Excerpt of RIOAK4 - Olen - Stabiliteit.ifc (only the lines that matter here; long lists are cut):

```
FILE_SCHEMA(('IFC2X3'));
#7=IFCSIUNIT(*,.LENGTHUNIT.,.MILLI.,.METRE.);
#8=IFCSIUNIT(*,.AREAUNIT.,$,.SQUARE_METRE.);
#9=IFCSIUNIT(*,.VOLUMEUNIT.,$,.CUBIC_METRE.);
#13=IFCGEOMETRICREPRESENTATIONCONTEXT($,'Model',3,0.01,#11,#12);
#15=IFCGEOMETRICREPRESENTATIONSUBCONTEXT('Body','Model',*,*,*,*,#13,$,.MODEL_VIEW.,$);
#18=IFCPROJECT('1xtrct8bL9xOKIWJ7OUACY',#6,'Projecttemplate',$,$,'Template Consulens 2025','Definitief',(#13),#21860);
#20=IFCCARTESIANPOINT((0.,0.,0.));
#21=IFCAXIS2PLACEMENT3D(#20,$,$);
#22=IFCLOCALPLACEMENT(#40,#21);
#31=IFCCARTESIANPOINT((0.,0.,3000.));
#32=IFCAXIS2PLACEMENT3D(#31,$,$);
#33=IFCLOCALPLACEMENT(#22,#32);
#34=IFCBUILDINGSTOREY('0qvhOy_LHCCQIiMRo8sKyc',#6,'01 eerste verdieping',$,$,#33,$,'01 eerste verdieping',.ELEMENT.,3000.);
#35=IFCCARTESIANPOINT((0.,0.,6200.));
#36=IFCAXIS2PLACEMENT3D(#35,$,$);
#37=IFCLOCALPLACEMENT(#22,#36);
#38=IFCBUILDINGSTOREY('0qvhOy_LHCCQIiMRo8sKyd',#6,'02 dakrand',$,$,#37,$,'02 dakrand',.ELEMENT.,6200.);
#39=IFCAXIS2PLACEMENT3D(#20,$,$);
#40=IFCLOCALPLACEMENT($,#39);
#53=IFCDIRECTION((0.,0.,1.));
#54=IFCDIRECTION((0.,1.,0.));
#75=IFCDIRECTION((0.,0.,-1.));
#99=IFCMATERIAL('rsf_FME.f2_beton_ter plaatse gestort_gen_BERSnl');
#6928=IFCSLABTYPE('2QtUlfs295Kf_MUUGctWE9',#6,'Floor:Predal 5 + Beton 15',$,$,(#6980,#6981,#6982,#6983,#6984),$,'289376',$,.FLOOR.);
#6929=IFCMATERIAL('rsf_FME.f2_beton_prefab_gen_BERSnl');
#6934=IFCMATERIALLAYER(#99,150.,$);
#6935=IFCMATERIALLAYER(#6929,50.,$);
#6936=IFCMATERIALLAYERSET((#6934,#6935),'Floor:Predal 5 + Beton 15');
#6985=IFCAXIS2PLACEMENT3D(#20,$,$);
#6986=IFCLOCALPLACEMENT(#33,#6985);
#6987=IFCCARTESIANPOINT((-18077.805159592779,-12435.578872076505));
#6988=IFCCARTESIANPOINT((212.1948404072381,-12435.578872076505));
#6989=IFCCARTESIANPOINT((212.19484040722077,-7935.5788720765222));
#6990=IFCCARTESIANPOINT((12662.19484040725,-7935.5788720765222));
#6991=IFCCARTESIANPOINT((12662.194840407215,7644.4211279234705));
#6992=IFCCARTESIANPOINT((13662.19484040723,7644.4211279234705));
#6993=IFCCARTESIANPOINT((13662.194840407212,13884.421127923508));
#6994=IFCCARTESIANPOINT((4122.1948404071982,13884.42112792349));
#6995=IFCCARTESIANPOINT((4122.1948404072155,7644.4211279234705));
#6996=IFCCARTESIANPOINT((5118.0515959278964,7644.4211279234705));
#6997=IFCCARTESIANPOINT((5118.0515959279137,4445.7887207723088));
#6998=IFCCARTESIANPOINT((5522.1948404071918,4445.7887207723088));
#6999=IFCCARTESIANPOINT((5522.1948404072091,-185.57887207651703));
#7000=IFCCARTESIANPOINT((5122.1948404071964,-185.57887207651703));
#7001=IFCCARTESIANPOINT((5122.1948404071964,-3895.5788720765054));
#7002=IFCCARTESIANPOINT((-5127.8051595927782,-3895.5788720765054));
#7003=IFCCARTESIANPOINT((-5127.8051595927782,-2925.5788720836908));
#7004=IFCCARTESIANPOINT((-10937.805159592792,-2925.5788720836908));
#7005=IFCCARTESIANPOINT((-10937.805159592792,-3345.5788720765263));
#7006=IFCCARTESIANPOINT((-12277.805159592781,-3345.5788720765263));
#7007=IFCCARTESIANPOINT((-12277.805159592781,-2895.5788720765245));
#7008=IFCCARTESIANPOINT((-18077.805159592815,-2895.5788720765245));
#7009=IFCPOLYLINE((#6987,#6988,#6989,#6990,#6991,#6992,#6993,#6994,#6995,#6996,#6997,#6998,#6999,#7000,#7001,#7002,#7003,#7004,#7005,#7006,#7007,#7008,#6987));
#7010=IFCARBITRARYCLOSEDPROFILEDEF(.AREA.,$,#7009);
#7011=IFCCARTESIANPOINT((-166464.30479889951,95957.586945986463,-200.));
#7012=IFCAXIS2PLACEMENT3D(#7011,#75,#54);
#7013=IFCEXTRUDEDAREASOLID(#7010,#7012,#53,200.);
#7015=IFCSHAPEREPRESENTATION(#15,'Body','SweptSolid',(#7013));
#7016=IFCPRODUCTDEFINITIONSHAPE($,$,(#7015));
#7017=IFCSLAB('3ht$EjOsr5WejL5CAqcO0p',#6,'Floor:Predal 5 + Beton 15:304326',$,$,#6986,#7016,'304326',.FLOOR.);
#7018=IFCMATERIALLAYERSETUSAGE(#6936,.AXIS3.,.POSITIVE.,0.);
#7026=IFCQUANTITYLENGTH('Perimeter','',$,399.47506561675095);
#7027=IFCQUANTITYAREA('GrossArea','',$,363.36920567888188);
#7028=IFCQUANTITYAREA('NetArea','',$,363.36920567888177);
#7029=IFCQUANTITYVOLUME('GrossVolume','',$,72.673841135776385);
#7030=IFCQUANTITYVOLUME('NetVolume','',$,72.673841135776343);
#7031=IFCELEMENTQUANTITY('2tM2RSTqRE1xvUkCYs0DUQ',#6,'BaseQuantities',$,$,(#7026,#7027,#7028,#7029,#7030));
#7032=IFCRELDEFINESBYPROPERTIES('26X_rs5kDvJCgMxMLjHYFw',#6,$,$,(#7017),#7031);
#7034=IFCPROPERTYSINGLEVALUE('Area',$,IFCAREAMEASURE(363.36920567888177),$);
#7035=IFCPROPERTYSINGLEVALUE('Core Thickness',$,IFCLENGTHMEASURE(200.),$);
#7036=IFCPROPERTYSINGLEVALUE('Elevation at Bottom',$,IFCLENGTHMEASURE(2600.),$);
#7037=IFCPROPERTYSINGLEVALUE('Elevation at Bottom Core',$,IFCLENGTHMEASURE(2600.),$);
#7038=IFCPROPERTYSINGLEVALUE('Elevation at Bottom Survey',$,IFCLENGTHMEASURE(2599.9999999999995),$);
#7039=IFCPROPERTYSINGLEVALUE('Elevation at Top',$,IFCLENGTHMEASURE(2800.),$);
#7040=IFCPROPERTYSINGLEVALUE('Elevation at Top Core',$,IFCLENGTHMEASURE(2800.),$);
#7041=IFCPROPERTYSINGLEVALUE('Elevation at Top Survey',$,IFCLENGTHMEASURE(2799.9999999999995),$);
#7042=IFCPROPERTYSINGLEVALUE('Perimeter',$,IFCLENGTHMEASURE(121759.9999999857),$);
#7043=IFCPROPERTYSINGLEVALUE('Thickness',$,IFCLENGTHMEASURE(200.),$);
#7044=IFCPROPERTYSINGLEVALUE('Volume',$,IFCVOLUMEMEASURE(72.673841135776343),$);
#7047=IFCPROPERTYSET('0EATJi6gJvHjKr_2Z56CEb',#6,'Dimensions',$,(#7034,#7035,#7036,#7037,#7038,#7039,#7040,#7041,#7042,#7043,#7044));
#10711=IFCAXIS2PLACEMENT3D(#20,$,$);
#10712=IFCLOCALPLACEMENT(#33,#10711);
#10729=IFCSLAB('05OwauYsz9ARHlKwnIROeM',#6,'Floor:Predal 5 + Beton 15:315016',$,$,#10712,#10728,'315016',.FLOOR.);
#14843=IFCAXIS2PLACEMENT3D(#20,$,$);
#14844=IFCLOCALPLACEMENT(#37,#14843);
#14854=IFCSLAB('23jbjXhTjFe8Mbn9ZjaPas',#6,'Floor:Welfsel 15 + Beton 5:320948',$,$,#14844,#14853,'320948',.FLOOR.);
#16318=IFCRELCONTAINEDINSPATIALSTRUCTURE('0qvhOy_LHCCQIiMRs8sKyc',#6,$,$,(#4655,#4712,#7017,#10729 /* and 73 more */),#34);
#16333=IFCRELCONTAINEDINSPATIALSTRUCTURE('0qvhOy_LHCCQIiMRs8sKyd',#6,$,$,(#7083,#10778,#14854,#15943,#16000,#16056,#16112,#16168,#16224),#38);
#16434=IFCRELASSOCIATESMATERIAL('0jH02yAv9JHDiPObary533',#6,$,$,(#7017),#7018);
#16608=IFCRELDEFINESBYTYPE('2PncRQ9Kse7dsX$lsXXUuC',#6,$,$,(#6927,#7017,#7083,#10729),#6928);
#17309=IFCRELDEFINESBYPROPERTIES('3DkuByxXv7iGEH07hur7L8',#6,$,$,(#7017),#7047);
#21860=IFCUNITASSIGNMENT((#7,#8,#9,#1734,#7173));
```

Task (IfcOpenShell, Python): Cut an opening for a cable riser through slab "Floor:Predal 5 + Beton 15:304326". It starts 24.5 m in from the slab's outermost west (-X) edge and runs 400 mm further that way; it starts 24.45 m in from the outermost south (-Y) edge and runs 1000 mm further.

```python
import numpy as np
import ifcopenshell
import ifcopenshell.api.feature
import ifcopenshell.api.geometry
import ifcopenshell.api.pset
import ifcopenshell.api.root
import ifcopenshell.geom
import ifcopenshell.util.element
import ifcopenshell.util.placement
import ifcopenshell.util.representation
import ifcopenshell.util.shape
import ifcopenshell.util.unit

model = ifcopenshell.open("RIOAK4 - Olen - Stabiliteit.ifc")
unit_scale = ifcopenshell.util.unit.calculate_unit_scale(model)
area_scale = ifcopenshell.util.unit.calculate_unit_scale(model, "AREAUNIT")
volume_scale = ifcopenshell.util.unit.calculate_unit_scale(model, "VOLUMEUNIT")
settings = ifcopenshell.geom.settings()


def volume(element):
    """Net volume in cubic metres, openings subtracted."""
    shape = ifcopenshell.geom.create_shape(settings, element)
    return ifcopenshell.util.shape.get_volume(shape.geometry)


slab = model.by_guid("3ht$EjOsr5WejL5CAqcO0p")
before = volume(slab)

# Extent in the slab's own axes, in metres. The edges named are its -X and -Y sides.
slab_shape = ifcopenshell.geom.create_shape(settings, slab)
vertices = ifcopenshell.util.shape.get_vertices(slab_shape.geometry)
x_min, y_min, bottom = vertices.min(axis=0)
top = vertices[:, 2].max()

opening = ifcopenshell.api.root.create_entity(model, ifc_class="IfcOpeningElement", name="Cable riser opening")
context = ifcopenshell.util.representation.get_context(model, "Model", "Body", "MODEL_VIEW")
width, depth = 0.4, 1
outline = [(0.0, 0.0), (width, 0.0), (width, depth), (0.0, depth), (0.0, 0.0)]
# Overshoot both faces by 50 mm so the cut is clean.
shape = ifcopenshell.api.geometry.add_slab_representation(
    model, context=context, depth=top - bottom + 0.1, polyline=outline
)
ifcopenshell.api.geometry.assign_representation(model, product=opening, representation=shape)

matrix = ifcopenshell.util.placement.get_local_placement(slab.ObjectPlacement)
matrix[:, 3] = matrix @ np.append(np.array([x_min + 24.5, y_min + 24.45, bottom - 0.05]) / unit_scale, 1.0)
ifcopenshell.api.geometry.edit_object_placement(model, product=opening, matrix=matrix, is_si=False)
ifcopenshell.api.feature.add_feature(model, feature=opening, element=slab)

after = volume(slab)

# Update the slab's stored quantities.
qto = model.by_id(ifcopenshell.util.element.get_pset(slab, "BaseQuantities", should_inherit=False)["id"])
ifcopenshell.api.pset.edit_qto(model, qto=qto, properties={
    "NetArea": after / (top - bottom) / area_scale,
    "NetVolume": after / volume_scale,
})
pset = model.by_id(ifcopenshell.util.element.get_pset(slab, "Dimensions", should_inherit=False)["id"])
ifcopenshell.api.pset.edit_pset(model, pset=pset, properties={
    "Area": model.create_entity("IfcAreaMeasure", after / (top - bottom) / area_scale),
    "Volume": model.create_entity("IfcVolumeMeasure", after / volume_scale),
})

print(f"slab volume {before:.3f} -> {after:.3f} m3")

model.write("RIOAK4 - Olen - Stabiliteit_updated.ifc")
```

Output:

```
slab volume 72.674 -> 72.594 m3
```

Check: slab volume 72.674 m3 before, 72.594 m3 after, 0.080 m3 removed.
